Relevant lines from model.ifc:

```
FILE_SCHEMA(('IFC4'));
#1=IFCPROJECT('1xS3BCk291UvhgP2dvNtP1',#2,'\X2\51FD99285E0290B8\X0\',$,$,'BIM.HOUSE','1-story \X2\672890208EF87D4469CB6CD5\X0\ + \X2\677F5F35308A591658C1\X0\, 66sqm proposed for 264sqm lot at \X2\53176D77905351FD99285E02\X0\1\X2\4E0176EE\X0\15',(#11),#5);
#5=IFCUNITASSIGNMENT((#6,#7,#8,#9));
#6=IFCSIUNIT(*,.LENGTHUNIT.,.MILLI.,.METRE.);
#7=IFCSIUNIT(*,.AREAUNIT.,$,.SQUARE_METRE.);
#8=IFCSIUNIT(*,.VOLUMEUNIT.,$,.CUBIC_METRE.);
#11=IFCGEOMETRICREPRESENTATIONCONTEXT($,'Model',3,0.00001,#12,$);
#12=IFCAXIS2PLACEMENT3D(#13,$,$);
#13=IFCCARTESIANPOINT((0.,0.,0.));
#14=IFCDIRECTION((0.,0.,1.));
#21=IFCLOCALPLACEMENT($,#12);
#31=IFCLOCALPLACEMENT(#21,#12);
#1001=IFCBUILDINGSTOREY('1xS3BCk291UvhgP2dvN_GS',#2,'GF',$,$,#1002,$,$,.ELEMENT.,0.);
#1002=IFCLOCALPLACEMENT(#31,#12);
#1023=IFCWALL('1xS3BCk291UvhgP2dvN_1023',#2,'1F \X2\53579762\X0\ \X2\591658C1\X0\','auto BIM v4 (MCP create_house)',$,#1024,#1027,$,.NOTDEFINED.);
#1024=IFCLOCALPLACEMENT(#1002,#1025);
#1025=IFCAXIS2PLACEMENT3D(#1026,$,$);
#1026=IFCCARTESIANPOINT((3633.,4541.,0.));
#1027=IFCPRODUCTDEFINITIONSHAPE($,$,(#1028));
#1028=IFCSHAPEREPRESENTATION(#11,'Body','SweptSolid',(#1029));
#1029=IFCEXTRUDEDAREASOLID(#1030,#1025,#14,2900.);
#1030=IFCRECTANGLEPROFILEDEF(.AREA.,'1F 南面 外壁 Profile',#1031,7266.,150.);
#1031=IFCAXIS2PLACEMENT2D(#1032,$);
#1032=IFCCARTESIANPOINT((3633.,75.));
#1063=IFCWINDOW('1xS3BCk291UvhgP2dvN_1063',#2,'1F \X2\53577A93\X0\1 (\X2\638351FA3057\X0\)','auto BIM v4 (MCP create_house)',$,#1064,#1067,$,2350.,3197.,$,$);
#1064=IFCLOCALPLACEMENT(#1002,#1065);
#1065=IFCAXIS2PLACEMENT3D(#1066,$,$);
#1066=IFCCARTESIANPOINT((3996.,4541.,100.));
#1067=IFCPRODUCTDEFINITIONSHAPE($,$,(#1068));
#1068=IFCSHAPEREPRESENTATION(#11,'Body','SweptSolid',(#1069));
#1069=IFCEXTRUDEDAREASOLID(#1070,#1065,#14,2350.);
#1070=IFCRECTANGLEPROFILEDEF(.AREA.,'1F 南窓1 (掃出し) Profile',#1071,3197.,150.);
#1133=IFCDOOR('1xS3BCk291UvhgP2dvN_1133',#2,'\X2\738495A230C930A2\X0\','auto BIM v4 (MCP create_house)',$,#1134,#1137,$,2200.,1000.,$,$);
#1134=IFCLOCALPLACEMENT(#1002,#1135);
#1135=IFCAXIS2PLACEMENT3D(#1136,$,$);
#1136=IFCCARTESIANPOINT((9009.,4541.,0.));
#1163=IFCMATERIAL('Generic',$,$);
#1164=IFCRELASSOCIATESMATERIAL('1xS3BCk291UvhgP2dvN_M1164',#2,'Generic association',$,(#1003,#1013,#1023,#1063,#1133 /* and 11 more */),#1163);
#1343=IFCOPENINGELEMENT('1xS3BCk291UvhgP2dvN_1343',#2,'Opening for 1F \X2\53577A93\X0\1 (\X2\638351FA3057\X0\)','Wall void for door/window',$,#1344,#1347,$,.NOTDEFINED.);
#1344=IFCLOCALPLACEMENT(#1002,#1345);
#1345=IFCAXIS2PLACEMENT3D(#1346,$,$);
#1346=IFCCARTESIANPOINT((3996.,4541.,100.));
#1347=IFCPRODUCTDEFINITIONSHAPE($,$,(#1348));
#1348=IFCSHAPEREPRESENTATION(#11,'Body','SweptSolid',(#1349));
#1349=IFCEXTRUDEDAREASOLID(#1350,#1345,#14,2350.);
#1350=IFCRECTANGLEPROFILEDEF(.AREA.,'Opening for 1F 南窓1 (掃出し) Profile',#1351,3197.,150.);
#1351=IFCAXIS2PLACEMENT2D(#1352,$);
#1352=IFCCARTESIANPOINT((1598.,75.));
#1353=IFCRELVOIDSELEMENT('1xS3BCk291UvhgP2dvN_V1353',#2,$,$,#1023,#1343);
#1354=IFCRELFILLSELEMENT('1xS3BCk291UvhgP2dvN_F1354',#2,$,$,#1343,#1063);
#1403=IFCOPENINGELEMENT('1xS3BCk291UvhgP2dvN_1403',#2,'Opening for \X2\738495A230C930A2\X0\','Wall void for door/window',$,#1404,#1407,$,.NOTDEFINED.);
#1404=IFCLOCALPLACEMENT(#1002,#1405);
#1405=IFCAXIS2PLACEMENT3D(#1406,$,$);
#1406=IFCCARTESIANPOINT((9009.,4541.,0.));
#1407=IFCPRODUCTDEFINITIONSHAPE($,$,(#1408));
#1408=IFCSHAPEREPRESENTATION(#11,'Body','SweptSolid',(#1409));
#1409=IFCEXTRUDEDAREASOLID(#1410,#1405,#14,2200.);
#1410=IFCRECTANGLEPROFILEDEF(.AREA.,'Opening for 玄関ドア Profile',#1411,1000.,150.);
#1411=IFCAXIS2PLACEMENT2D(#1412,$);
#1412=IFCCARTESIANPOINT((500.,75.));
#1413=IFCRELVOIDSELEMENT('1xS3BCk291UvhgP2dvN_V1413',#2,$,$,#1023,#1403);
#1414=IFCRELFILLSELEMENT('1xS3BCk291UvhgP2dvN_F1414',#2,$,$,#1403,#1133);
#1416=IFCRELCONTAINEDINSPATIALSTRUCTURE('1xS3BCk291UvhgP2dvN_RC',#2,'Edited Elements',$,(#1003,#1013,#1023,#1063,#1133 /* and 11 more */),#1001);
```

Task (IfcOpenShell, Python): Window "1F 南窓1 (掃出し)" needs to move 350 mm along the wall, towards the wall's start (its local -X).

```python
import ifcopenshell
import ifcopenshell.api.geometry
import ifcopenshell.util.placement
import ifcopenshell.util.unit

model = ifcopenshell.open("model.ifc")
unit_scale = ifcopenshell.util.unit.calculate_unit_scale(model)

window = model.by_guid("1xS3BCk291UvhgP2dvN_1063")
opening = window.FillsVoids[0].RelatingOpeningElement
wall = opening.VoidsElements[0].RelatingBuildingElement

wall_matrix = ifcopenshell.util.placement.get_local_placement(wall.ObjectPlacement)
shift = wall_matrix[:3, 0] * -0.35 / unit_scale
before = ifcopenshell.util.placement.get_local_placement(window.ObjectPlacement)[:3, 3].copy()

# The window is not placed relative to its opening, so move both.
for product in (opening, window):
    matrix = ifcopenshell.util.placement.get_local_placement(product.ObjectPlacement)
    matrix[:3, 3] += shift
    ifcopenshell.api.geometry.edit_object_placement(model, product=product, matrix=matrix, is_si=False)

after = ifcopenshell.util.placement.get_local_placement(window.ObjectPlacement)[:3, 3]
print("window moved by", (after - before).round(3) + 0.0)

model.write("model_rev.ifc")
```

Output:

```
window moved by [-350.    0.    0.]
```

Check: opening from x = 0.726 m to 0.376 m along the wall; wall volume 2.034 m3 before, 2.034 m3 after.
